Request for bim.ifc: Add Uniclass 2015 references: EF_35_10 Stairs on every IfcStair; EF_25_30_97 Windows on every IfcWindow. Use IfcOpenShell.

First a look at what the model holds.

```python
import ifcopenshell

model = ifcopenshell.open("bim.ifc")
print(model.schema)
print("classifications:", [c.Name for c in model.by_type("IfcClassification")])
for ifc_class in ("IfcDoor", "IfcRoof", "IfcStair", "IfcWall", "IfcWindow"):
    print(ifc_class, len(model.by_type(ifc_class)))
```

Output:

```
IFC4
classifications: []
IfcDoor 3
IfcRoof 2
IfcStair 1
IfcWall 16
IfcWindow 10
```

```python
import ifcopenshell
import ifcopenshell.api.classification

model = ifcopenshell.open("bim.ifc")

system = ifcopenshell.api.classification.add_classification(model, classification="Uniclass 2015")

codes = {
    "IfcStair": ("EF_35_10", "Stairs"),
    "IfcWindow": ("EF_25_30_97", "Windows"),
}
for ifc_class, (code, name) in codes.items():
    products = model.by_type(ifc_class)
    ifcopenshell.api.classification.add_reference(
        model, products=products, classification=system, identification=code, name=name
    )
    print(code, len(products))

model.write("bim_rev.ifc")
```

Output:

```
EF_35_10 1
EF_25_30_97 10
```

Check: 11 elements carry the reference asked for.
